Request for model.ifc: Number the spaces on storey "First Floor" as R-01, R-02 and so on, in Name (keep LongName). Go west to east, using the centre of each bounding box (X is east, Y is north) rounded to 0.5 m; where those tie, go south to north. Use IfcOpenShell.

First a look at what the model holds.

```python
import ifcopenshell
import ifcopenshell.util.element
import ifcopenshell.util.placement

model = ifcopenshell.open("model.ifc")
print(model.schema)
storey = next(s for s in model.by_type("IfcBuildingStorey") if s.Name == "First Floor")
spaces = [e for e in ifcopenshell.util.element.get_decomposition(storey) if e.is_a("IfcSpace")]
for e in sorted(spaces, key=lambda e: e.id()):
    origin = ifcopenshell.util.placement.get_local_placement(e.ObjectPlacement)[:3, 3]
    print(e.id(), e.Name, e.LongName, origin.round(2) + 0.0, sep=" | ")
```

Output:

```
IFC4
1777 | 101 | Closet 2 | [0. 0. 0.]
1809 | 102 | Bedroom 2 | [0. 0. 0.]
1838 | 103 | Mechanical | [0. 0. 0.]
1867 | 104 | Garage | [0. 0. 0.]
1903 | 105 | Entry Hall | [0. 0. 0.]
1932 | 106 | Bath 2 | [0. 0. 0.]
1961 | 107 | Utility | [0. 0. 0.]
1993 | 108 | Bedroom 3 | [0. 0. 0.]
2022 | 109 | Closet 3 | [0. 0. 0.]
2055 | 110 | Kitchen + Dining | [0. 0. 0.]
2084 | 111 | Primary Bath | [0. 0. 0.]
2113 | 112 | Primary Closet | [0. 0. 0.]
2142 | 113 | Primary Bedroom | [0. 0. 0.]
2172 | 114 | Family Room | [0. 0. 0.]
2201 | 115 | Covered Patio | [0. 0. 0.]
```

```python
import ifcopenshell
import ifcopenshell.geom
import ifcopenshell.util.element
import ifcopenshell.util.shape

model = ifcopenshell.open("model.ifc")
settings = ifcopenshell.geom.settings()
settings.set("use-world-coords", True)


def centre(element):
    shape = ifcopenshell.geom.create_shape(settings, element)
    return ifcopenshell.util.shape.get_bbox_centroid(shape.geometry)


storey = next(s for s in model.by_type("IfcBuildingStorey") if s.Name == "First Floor")
spaces = [e for e in ifcopenshell.util.element.get_decomposition(storey) if e.is_a("IfcSpace")]

# Insertion points can sit at a corner or the storey origin, so sort by the geometry (in metres).
centres = {e: centre(e) for e in spaces}
spaces.sort(key=lambda e: (round(centres[e][0] / 0.5), centres[e][1]))

for i, e in enumerate(spaces, start=1):
    number = f"R-{i:02d}"
    e.Name = number
    print(e.id(), number)

model.write("model_v2.ifc")
```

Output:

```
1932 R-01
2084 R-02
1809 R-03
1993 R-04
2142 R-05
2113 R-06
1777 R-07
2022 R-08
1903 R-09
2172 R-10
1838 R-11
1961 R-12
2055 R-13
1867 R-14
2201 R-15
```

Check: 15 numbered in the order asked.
